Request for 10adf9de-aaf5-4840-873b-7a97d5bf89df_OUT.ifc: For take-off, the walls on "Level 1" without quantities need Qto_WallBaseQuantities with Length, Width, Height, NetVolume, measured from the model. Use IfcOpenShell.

First a look at what the model holds.

```python
import ifcopenshell
import ifcopenshell.util.element
import ifcopenshell.util.unit

model = ifcopenshell.open("10adf9de-aaf5-4840-873b-7a97d5bf89df_OUT.ifc")
print(model.schema)
for unit_type in ("LENGTHUNIT", "AREAUNIT", "VOLUMEUNIT"):
    print(unit_type, ifcopenshell.util.unit.calculate_unit_scale(model, unit_type))
storey = next(s for s in model.by_type("IfcBuildingStorey") if s.Name == "Level 1")
walls = [e for e in ifcopenshell.util.element.get_decomposition(storey) if e.is_a("IfcWall")]
for e in sorted(walls, key=lambda e: e.id()):
    print(e.id(), e.is_a(), e.Name, list(ifcopenshell.util.element.get_psets(e, qtos_only=True)), sep=" | ")
```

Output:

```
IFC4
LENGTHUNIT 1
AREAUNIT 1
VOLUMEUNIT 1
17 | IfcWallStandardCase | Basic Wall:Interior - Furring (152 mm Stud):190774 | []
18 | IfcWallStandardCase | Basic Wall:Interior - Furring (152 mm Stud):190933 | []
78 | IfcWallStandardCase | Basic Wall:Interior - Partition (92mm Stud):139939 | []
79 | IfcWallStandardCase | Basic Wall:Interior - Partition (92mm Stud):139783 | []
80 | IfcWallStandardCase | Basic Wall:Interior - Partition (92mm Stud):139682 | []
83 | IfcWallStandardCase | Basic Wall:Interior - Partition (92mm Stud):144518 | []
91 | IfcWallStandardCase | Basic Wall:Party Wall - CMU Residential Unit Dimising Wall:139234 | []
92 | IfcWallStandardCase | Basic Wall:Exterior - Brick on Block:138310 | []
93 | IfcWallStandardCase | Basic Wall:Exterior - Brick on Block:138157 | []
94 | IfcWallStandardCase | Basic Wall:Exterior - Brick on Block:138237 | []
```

```python
import ifcopenshell
import ifcopenshell.api.pset
import ifcopenshell.geom
import ifcopenshell.util.element
import ifcopenshell.util.shape
import ifcopenshell.util.unit

model = ifcopenshell.open("10adf9de-aaf5-4840-873b-7a97d5bf89df_OUT.ifc")
unit_scale = ifcopenshell.util.unit.calculate_unit_scale(model)
volume_scale = ifcopenshell.util.unit.calculate_unit_scale(model, "VOLUMEUNIT")
settings = ifcopenshell.geom.settings()

storey = next(s for s in model.by_type("IfcBuildingStorey") if s.Name == "Level 1")
walls = [e for e in ifcopenshell.util.element.get_decomposition(storey) if e.is_a("IfcWall")]

for e in sorted(walls, key=lambda e: e.id()):
    if ifcopenshell.util.element.get_psets(e, qtos_only=True, should_inherit=False):
        continue
    # Geometry comes back in metres, in the element's own axes.
    shape = ifcopenshell.geom.create_shape(settings, e)
    values = {
        "Length": ifcopenshell.util.shape.get_x(shape.geometry) / unit_scale,
        "Width": ifcopenshell.util.shape.get_y(shape.geometry) / unit_scale,
        "Height": ifcopenshell.util.shape.get_z(shape.geometry) / unit_scale,
        "NetVolume": ifcopenshell.util.shape.get_volume(shape.geometry) / volume_scale,
    }
    qto = ifcopenshell.api.pset.add_qto(model, product=e, name="Qto_WallBaseQuantities")
    ifcopenshell.api.pset.edit_qto(model, qto=qto, properties=values)
    print(e.id(), {k: round(v, 3) for k, v in values.items()})

model.write("10adf9de-aaf5-4840-873b-7a97d5bf89df_OUT-out.ifc")
```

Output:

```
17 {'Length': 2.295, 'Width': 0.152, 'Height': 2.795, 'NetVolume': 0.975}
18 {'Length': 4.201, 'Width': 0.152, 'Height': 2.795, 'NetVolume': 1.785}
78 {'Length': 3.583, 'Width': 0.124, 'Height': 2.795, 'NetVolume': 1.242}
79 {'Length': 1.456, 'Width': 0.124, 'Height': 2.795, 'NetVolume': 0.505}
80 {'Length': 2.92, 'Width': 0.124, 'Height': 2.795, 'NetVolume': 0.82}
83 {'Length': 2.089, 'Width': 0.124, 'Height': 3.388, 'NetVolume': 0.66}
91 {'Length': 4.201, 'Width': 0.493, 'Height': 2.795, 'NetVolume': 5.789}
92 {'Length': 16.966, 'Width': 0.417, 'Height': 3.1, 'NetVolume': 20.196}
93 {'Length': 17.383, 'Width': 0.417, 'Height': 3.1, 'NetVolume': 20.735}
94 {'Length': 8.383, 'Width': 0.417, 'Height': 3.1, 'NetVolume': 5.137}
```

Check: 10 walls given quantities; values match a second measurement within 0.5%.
